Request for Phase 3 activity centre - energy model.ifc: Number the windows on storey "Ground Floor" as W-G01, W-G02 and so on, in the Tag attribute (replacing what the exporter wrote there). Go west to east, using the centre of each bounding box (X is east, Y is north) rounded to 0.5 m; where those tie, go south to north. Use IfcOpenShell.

First a look at what the model holds.

```python
import ifcopenshell
import ifcopenshell.util.element
import ifcopenshell.util.placement

model = ifcopenshell.open("Phase 3 activity centre - energy model.ifc")
print(model.schema)
storey = next(s for s in model.by_type("IfcBuildingStorey") if s.Name == "Ground Floor")
windows = [e for e in ifcopenshell.util.element.get_decomposition(storey) if e.is_a("IfcWindow")]
for e in sorted(windows, key=lambda e: e.id()):
    origin = ifcopenshell.util.placement.get_local_placement(e.ObjectPlacement)[:3, 3]
    print(e.id(), e.Tag, e.Name, origin.round(2) + 0.0, sep=" | ")
```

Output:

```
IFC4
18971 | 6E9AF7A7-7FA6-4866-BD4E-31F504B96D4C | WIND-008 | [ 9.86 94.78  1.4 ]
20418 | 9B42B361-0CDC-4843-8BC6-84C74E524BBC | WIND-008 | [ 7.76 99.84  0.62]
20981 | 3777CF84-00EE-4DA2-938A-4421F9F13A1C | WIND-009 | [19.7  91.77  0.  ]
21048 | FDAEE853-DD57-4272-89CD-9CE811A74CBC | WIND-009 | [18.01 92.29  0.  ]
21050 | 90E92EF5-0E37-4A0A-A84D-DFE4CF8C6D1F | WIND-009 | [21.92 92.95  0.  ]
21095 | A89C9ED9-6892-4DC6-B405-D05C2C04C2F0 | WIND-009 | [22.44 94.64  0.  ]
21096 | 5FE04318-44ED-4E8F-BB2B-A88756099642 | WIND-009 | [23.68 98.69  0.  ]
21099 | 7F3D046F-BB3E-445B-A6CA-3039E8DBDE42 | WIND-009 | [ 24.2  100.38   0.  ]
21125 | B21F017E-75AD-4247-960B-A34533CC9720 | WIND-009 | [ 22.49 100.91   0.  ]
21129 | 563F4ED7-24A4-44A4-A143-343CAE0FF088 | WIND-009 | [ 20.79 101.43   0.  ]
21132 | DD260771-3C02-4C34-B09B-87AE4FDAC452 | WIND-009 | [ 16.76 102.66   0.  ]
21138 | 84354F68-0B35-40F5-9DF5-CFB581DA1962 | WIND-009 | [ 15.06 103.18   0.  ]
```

```python
import ifcopenshell
import ifcopenshell.geom
import ifcopenshell.util.element
import ifcopenshell.util.shape

model = ifcopenshell.open("Phase 3 activity centre - energy model.ifc")
settings = ifcopenshell.geom.settings()
settings.set("use-world-coords", True)


def centre(element):
    shape = ifcopenshell.geom.create_shape(settings, element)
    return ifcopenshell.util.shape.get_bbox_centroid(shape.geometry)


storey = next(s for s in model.by_type("IfcBuildingStorey") if s.Name == "Ground Floor")
windows = [e for e in ifcopenshell.util.element.get_decomposition(storey) if e.is_a("IfcWindow")]

# Insertion points can sit at a corner or the storey origin, so sort by the geometry (in metres).
centres = {e: centre(e) for e in windows}
windows.sort(key=lambda e: (round(centres[e][0] / 0.5), centres[e][1]))

for i, e in enumerate(windows, start=1):
    number = f"W-G{i:02d}"
    e.Tag = number
    print(e.id(), number)

model.write("Phase 3 activity centre - energy model_rev.ifc")
```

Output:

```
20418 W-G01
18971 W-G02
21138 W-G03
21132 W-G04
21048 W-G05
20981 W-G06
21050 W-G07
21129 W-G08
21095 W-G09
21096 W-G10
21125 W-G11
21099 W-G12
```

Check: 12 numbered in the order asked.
